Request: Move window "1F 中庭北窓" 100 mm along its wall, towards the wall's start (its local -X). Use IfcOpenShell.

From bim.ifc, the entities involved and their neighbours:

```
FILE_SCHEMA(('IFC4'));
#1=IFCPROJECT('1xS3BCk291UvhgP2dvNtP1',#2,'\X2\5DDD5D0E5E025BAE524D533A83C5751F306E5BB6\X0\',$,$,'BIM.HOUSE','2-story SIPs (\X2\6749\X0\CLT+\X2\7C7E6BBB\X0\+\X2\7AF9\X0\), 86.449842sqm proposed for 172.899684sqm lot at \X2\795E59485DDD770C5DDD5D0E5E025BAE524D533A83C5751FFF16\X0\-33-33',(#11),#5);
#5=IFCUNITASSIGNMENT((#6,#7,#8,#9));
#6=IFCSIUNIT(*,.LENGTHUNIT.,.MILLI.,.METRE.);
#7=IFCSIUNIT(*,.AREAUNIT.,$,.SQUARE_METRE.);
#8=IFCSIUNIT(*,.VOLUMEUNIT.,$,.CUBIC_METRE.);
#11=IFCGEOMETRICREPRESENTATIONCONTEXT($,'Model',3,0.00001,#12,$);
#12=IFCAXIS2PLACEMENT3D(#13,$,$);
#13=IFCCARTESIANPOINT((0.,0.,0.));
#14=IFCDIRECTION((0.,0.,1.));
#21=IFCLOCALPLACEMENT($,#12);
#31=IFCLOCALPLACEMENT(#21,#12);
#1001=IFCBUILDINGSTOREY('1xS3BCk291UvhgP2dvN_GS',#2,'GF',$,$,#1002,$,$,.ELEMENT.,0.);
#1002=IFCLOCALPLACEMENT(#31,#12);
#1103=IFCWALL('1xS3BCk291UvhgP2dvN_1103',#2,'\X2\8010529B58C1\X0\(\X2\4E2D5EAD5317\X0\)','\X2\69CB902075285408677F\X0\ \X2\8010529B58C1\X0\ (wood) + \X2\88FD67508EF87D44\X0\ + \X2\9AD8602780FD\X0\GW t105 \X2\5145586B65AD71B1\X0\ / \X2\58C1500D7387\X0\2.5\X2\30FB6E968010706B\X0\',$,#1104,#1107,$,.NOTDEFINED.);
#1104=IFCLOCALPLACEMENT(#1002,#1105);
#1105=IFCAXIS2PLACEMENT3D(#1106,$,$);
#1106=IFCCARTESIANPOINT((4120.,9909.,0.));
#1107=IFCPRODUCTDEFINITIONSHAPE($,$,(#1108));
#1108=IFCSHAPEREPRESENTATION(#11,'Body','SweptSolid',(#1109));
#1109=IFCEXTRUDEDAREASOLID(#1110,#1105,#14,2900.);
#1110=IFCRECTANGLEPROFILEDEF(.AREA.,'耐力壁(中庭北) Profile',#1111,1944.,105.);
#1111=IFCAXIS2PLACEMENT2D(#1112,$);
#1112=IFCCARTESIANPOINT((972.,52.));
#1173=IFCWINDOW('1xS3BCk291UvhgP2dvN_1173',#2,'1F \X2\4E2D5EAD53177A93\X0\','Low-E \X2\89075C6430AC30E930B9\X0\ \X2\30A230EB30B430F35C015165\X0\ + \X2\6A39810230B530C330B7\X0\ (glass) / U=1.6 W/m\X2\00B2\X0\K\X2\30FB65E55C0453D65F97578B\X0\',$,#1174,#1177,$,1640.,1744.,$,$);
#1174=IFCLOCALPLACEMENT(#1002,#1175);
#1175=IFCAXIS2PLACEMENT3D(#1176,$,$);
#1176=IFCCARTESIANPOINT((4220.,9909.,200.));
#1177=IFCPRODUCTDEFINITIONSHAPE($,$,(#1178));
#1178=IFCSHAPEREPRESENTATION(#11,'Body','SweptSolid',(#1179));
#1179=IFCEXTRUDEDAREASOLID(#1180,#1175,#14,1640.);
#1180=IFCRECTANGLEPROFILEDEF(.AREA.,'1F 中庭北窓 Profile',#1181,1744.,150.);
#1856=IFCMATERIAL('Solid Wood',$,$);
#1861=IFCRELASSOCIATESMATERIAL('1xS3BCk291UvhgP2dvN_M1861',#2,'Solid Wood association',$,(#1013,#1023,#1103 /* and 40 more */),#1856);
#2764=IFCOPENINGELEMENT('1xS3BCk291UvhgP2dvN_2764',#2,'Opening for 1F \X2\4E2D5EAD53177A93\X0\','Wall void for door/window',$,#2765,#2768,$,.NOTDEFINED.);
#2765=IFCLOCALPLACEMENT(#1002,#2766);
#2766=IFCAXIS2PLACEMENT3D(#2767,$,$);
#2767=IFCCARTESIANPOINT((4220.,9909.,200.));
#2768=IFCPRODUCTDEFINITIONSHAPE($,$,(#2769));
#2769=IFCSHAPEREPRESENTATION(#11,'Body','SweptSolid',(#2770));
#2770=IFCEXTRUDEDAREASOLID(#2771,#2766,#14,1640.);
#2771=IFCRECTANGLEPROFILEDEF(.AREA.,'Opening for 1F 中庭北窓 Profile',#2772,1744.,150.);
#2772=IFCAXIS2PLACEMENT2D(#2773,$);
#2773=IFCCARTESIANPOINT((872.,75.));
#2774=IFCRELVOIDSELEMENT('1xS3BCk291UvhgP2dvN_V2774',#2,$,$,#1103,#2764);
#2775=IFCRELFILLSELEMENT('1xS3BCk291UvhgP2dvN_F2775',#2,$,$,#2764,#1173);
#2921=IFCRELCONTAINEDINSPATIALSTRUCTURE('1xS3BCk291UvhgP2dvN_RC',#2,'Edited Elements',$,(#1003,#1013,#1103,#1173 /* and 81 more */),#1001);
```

```python
import ifcopenshell
import ifcopenshell.api.geometry
import ifcopenshell.util.placement
import ifcopenshell.util.unit

model = ifcopenshell.open("bim.ifc")
unit_scale = ifcopenshell.util.unit.calculate_unit_scale(model)

window = model.by_id(1173)
opening = window.FillsVoids[0].RelatingOpeningElement
wall = opening.VoidsElements[0].RelatingBuildingElement

wall_matrix = ifcopenshell.util.placement.get_local_placement(wall.ObjectPlacement)
shift = wall_matrix[:3, 0] * -0.1 / unit_scale
before = ifcopenshell.util.placement.get_local_placement(window.ObjectPlacement)[:3, 3].copy()

# The window is not placed relative to its opening, so move both.
for product in (opening, window):
    matrix = ifcopenshell.util.placement.get_local_placement(product.ObjectPlacement)
    matrix[:3, 3] += shift
    ifcopenshell.api.geometry.edit_object_placement(model, product=product, matrix=matrix, is_si=False)

after = ifcopenshell.util.placement.get_local_placement(window.ObjectPlacement)[:3, 3]
print("window moved by", (after - before).round(3) + 0.0)

model.write("bim_v2.ifc")
```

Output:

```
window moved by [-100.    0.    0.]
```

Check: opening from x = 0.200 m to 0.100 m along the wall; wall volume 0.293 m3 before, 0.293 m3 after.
